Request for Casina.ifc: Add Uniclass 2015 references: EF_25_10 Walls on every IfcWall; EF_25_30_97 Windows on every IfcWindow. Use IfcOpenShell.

First a look at what the model holds.

```python
import ifcopenshell

model = ifcopenshell.open("Casina.ifc")
print(model.schema)
print("classifications:", [c.Name for c in model.by_type("IfcClassification")])
for ifc_class in ("IfcDoor", "IfcRoof", "IfcStair", "IfcWall", "IfcWindow"):
    print(ifc_class, len(model.by_type(ifc_class)))
```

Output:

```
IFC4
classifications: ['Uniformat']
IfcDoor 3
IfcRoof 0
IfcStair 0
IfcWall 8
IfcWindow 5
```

```python
import ifcopenshell
import ifcopenshell.api.classification

model = ifcopenshell.open("Casina.ifc")

system = ifcopenshell.api.classification.add_classification(model, classification="Uniclass 2015")

codes = {
    "IfcWall": ("EF_25_10", "Walls"),
    "IfcWindow": ("EF_25_30_97", "Windows"),
}
for ifc_class, (code, name) in codes.items():
    products = model.by_type(ifc_class)
    ifcopenshell.api.classification.add_reference(
        model, products=products, classification=system, identification=code, name=name
    )
    print(code, len(products))

model.write("Casina_rev.ifc")
```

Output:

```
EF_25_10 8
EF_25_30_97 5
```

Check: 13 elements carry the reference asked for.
